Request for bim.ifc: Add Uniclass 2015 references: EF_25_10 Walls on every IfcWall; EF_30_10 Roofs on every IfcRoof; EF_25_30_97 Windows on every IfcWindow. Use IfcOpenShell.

First a look at what the model holds.

```python
import ifcopenshell

model = ifcopenshell.open("bim.ifc")
print(model.schema)
print("classifications:", [c.Name for c in model.by_type("IfcClassification")])
for ifc_class in ("IfcDoor", "IfcRoof", "IfcStair", "IfcWall", "IfcWindow"):
    print(ifc_class, len(model.by_type(ifc_class)))
```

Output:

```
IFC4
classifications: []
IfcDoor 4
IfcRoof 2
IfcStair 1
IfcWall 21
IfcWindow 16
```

```python
import ifcopenshell
import ifcopenshell.api.classification

model = ifcopenshell.open("bim.ifc")

system = ifcopenshell.api.classification.add_classification(model, classification="Uniclass 2015")

codes = {
    "IfcWall": ("EF_25_10", "Walls"),
    "IfcRoof": ("EF_30_10", "Roofs"),
    "IfcWindow": ("EF_25_30_97", "Windows"),
}
for ifc_class, (code, name) in codes.items():
    products = model.by_type(ifc_class)
    ifcopenshell.api.classification.add_reference(
        model, products=products, classification=system, identification=code, name=name
    )
    print(code, len(products))

model.write("bim_edited.ifc")
```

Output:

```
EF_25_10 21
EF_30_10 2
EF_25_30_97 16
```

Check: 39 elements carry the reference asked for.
